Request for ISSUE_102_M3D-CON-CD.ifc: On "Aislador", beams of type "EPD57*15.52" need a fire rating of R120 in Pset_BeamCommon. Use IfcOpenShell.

First a look at what the model holds.

```python
import ifcopenshell
import ifcopenshell.util.element

model = ifcopenshell.open("ISSUE_102_M3D-CON-CD.ifc")
print(model.schema)
storey = next(s for s in model.by_type("IfcBuildingStorey") if s.Name == "Aislador")
beams = [e for e in ifcopenshell.util.element.get_decomposition(storey) if e.is_a("IfcBeam")]
seen = {}
for e in beams:
    element_type = ifcopenshell.util.element.get_type(e)
    key = (element_type.Name if element_type != e and element_type else None, ifcopenshell.util.element.get_pset(e, "Pset_BeamCommon", "FireRating"))
    seen[key] = seen.get(key, 0) + 1
for (name, value), count in sorted(seen.items(), key=str):
    print(count, "x", name, "|", value)
```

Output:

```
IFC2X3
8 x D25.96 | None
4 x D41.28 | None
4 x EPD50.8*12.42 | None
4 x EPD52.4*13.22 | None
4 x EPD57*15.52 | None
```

```python
import ifcopenshell
import ifcopenshell.api.pset
import ifcopenshell.util.element

model = ifcopenshell.open("ISSUE_102_M3D-CON-CD.ifc")

storey = next(s for s in model.by_type("IfcBuildingStorey") if s.Name == "Aislador")
beams = [e for e in ifcopenshell.util.element.get_decomposition(storey) if e.is_a("IfcBeam")]

count = 0
for e in beams:
    element_type = ifcopenshell.util.element.get_type(e)
    if element_type in (None, e) or element_type.Name != "EPD57*15.52":
        continue
    found = ifcopenshell.util.element.get_pset(e, "Pset_BeamCommon", should_inherit=False)
    if found:
        pset = model.by_id(found["id"])
        if len(ifcopenshell.util.element.get_elements_by_pset(pset)) > 1:
            pset = ifcopenshell.api.pset.unshare_pset(model, products=[e], pset=pset)[0]
    else:
        pset = ifcopenshell.api.pset.add_pset(model, product=e, name="Pset_BeamCommon")
    ifcopenshell.api.pset.edit_pset(model, pset=pset, properties={"FireRating": "R120"})
    count += 1

print(count, "beams updated")

model.write("ISSUE_102_M3D-CON-CD_v2.ifc")
```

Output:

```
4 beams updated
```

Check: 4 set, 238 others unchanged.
